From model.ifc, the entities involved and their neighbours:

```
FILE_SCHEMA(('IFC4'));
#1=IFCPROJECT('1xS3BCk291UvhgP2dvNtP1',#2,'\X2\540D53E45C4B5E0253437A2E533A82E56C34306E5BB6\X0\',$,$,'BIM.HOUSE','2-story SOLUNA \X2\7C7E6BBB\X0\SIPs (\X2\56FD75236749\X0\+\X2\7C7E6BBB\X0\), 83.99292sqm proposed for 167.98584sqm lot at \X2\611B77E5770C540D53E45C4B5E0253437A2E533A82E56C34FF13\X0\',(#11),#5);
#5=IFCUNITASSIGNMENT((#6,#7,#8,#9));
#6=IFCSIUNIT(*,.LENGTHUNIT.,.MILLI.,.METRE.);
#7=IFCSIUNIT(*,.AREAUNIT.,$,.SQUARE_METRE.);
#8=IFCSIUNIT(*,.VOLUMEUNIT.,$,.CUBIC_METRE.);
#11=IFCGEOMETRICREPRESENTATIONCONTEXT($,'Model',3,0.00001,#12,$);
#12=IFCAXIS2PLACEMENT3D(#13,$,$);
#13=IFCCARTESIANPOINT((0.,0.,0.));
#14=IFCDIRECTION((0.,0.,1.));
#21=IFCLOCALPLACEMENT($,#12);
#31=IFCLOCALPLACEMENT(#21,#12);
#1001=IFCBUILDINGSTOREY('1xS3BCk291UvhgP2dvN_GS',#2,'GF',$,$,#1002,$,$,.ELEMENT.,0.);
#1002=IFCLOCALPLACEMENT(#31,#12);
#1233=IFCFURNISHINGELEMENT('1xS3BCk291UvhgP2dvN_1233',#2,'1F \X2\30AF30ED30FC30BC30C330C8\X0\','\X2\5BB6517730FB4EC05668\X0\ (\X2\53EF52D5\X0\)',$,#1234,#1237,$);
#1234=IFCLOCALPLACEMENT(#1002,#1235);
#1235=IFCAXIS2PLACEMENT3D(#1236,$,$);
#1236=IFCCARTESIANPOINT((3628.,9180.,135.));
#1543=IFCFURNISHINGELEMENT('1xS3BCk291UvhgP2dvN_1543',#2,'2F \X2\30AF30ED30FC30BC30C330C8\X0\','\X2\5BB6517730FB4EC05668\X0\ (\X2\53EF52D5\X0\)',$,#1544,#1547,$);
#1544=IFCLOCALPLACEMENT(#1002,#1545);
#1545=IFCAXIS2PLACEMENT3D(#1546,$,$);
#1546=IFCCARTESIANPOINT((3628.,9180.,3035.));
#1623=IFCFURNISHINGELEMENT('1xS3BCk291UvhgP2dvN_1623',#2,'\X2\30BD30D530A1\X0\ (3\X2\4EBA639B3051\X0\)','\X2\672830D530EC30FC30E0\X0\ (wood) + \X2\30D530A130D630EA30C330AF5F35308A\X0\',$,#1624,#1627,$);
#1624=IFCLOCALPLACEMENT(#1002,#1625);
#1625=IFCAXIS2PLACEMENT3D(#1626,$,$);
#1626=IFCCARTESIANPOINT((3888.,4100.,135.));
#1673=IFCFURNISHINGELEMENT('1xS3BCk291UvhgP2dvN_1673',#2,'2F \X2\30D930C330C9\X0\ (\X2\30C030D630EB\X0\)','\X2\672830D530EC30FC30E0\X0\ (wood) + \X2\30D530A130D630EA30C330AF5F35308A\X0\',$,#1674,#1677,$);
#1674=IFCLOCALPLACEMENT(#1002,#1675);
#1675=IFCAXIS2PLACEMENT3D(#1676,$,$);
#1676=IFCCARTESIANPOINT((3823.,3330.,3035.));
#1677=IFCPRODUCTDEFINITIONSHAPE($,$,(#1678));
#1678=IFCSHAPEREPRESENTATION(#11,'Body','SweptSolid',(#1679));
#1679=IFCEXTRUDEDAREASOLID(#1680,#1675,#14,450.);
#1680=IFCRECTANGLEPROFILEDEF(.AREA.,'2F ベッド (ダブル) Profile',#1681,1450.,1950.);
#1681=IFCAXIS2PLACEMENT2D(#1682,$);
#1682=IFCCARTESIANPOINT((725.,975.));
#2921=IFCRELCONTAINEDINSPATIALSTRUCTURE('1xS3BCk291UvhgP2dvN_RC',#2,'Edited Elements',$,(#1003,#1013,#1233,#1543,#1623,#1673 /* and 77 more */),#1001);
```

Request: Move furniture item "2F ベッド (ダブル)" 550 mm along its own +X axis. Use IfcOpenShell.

```python
import ifcopenshell
import ifcopenshell.api.geometry
import ifcopenshell.util.placement
import ifcopenshell.util.unit

model = ifcopenshell.open("model.ifc")
unit_scale = ifcopenshell.util.unit.calculate_unit_scale(model)

item = model.by_id(1673)
matrix = ifcopenshell.util.placement.get_local_placement(item.ObjectPlacement)
matrix[:3, 3] += matrix[:3, 0] * 0.55 / unit_scale
ifcopenshell.api.geometry.edit_object_placement(model, product=item, matrix=matrix, is_si=False)

print(ifcopenshell.util.placement.get_local_placement(item.ObjectPlacement).round(3) + 0.0)

model.write("model-out.ifc")
```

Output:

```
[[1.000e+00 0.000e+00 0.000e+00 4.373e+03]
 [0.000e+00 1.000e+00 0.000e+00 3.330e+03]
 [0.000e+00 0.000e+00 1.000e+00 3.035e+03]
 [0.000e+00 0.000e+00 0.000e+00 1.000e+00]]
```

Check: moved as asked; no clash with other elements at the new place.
